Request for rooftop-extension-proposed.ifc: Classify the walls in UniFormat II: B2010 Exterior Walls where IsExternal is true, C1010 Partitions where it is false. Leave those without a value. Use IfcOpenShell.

First a look at what the model holds.

```python
import ifcopenshell
import ifcopenshell.util.element

model = ifcopenshell.open("rooftop-extension-proposed.ifc")
print(model.schema)
print("classifications:", [c.Name for c in model.by_type("IfcClassification")])
values = [ifcopenshell.util.element.get_pset(e, "Pset_WallCommon", "IsExternal") for e in model.by_type("IfcWall")]
for value in (True, False, None):
    print("IsExternal", value, values.count(value))
```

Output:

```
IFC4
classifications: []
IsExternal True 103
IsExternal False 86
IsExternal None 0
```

```python
import ifcopenshell
import ifcopenshell.api.classification
import ifcopenshell.util.element

model = ifcopenshell.open("rooftop-extension-proposed.ifc")

system = ifcopenshell.api.classification.add_classification(model, classification="UniFormat II")

walls = model.by_type("IfcWall")
external = {e: ifcopenshell.util.element.get_pset(e, "Pset_WallCommon", "IsExternal") for e in walls}
for flag, code, name in ((True, "B2010", "Exterior Walls"), (False, "C1010", "Partitions")):
    products = [e for e in walls if external[e] is flag]
    ifcopenshell.api.classification.add_reference(
        model, products=products, classification=system, identification=code, name=name
    )
    print(code, len(products))

model.write("rooftop-extension-proposed_edited.ifc")
```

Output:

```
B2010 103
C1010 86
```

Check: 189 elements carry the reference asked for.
